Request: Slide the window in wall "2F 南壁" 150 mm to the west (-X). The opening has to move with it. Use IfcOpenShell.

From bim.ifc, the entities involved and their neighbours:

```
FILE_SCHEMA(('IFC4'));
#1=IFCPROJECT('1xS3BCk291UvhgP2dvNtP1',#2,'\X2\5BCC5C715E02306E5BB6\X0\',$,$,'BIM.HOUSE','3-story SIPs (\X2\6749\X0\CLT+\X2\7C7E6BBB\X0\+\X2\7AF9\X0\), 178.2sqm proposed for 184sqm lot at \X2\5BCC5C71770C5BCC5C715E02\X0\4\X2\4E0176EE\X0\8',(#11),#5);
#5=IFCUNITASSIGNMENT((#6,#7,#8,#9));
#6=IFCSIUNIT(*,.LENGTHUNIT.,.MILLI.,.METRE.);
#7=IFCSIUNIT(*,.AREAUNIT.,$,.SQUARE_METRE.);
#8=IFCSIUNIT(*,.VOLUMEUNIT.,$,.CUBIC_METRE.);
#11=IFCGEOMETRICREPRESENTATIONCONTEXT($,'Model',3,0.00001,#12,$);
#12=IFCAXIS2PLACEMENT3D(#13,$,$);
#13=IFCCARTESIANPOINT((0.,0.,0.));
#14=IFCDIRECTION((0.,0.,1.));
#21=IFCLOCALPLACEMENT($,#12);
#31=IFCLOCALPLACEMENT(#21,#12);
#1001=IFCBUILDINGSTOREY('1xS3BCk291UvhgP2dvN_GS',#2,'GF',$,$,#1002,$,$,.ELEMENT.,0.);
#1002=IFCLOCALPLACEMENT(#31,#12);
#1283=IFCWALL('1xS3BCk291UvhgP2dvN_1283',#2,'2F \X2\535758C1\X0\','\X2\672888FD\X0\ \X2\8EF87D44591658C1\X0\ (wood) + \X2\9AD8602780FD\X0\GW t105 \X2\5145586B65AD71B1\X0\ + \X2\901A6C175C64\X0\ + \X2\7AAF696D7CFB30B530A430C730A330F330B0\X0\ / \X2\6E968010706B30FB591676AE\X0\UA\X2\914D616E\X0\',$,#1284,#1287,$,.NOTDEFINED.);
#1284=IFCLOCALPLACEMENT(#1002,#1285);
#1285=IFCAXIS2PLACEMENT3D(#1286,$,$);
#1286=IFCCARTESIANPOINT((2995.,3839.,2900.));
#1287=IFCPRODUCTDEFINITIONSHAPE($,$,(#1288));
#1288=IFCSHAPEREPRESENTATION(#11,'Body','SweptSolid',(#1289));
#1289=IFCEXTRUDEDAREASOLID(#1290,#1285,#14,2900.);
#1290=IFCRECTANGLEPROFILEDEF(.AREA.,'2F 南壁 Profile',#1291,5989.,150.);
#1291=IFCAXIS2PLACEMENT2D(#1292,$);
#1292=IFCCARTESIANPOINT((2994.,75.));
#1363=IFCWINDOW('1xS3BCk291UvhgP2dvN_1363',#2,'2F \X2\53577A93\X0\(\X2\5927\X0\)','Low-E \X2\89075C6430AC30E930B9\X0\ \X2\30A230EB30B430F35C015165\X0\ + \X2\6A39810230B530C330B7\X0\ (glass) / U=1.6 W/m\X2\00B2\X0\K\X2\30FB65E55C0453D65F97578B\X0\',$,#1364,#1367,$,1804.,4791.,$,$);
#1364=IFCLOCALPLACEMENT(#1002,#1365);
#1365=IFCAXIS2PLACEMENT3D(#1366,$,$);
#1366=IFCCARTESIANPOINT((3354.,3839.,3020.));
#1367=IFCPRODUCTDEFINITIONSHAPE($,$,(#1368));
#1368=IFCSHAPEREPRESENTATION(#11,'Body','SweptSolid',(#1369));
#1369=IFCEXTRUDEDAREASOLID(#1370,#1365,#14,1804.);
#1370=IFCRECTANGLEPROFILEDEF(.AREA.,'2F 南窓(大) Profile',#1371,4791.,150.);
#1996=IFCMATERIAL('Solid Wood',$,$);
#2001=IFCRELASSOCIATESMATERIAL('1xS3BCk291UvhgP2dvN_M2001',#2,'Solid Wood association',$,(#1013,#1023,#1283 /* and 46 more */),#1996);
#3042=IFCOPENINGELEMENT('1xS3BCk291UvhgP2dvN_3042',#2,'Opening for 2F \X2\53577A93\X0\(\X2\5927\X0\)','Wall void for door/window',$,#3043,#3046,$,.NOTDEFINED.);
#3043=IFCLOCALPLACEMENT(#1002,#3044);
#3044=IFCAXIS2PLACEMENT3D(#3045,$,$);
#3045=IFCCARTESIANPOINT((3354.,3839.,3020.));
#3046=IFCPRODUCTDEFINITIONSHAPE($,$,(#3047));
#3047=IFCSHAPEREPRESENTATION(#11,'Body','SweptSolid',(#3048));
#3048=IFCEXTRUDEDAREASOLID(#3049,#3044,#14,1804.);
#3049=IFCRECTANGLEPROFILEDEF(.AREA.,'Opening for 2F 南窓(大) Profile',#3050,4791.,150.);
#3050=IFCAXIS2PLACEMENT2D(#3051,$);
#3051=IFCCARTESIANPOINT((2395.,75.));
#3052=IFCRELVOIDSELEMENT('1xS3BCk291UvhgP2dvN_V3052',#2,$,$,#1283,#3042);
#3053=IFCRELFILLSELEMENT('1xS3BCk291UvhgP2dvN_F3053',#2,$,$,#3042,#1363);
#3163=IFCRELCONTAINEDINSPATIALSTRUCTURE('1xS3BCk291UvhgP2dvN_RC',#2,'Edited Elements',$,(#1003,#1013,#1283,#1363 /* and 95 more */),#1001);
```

```python
import ifcopenshell
import ifcopenshell.api.geometry
import ifcopenshell.util.placement
import ifcopenshell.util.unit

model = ifcopenshell.open("bim.ifc")
unit_scale = ifcopenshell.util.unit.calculate_unit_scale(model)

window = model.by_id(1363)
opening = window.FillsVoids[0].RelatingOpeningElement
wall = opening.VoidsElements[0].RelatingBuildingElement

wall_matrix = ifcopenshell.util.placement.get_local_placement(wall.ObjectPlacement)
shift = wall_matrix[:3, 0] * -0.15 / unit_scale
before = ifcopenshell.util.placement.get_local_placement(window.ObjectPlacement)[:3, 3].copy()

# The window is not placed relative to its opening, so move both.
for product in (opening, window):
    matrix = ifcopenshell.util.placement.get_local_placement(product.ObjectPlacement)
    matrix[:3, 3] += shift
    ifcopenshell.api.geometry.edit_object_placement(model, product=product, matrix=matrix, is_si=False)

after = ifcopenshell.util.placement.get_local_placement(window.ObjectPlacement)[:3, 3]
print("window moved by", (after - before).round(3) + 0.0)

model.write("bim_updated.ifc")
```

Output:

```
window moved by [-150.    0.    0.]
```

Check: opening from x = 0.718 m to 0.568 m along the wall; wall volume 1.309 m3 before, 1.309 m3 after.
